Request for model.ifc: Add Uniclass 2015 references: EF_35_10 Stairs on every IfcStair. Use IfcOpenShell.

First a look at what the model holds.

```python
import ifcopenshell

model = ifcopenshell.open("model.ifc")
print(model.schema)
print("classifications:", [c.Name for c in model.by_type("IfcClassification")])
for ifc_class in ("IfcDoor", "IfcRoof", "IfcStair", "IfcWall", "IfcWindow"):
    print(ifc_class, len(model.by_type(ifc_class)))
```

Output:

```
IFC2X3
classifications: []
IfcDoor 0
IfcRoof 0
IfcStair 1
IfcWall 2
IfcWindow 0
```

```python
import ifcopenshell
import ifcopenshell.api.classification

model = ifcopenshell.open("model.ifc")

# IFC2X3 requires Source and Edition and has no link from the project to the system.
system = model.create_entity("IfcClassification", Source="NBS", Edition="2015", Name="Uniclass 2015")

codes = {
    "IfcStair": ("EF_35_10", "Stairs"),
}
for ifc_class, (code, name) in codes.items():
    products = model.by_type(ifc_class)
    ifcopenshell.api.classification.add_reference(
        model, products=products, classification=system, identification=code, name=name
    )
    print(code, len(products))

model.write("model_edited.ifc")
```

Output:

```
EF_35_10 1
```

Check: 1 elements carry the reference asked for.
